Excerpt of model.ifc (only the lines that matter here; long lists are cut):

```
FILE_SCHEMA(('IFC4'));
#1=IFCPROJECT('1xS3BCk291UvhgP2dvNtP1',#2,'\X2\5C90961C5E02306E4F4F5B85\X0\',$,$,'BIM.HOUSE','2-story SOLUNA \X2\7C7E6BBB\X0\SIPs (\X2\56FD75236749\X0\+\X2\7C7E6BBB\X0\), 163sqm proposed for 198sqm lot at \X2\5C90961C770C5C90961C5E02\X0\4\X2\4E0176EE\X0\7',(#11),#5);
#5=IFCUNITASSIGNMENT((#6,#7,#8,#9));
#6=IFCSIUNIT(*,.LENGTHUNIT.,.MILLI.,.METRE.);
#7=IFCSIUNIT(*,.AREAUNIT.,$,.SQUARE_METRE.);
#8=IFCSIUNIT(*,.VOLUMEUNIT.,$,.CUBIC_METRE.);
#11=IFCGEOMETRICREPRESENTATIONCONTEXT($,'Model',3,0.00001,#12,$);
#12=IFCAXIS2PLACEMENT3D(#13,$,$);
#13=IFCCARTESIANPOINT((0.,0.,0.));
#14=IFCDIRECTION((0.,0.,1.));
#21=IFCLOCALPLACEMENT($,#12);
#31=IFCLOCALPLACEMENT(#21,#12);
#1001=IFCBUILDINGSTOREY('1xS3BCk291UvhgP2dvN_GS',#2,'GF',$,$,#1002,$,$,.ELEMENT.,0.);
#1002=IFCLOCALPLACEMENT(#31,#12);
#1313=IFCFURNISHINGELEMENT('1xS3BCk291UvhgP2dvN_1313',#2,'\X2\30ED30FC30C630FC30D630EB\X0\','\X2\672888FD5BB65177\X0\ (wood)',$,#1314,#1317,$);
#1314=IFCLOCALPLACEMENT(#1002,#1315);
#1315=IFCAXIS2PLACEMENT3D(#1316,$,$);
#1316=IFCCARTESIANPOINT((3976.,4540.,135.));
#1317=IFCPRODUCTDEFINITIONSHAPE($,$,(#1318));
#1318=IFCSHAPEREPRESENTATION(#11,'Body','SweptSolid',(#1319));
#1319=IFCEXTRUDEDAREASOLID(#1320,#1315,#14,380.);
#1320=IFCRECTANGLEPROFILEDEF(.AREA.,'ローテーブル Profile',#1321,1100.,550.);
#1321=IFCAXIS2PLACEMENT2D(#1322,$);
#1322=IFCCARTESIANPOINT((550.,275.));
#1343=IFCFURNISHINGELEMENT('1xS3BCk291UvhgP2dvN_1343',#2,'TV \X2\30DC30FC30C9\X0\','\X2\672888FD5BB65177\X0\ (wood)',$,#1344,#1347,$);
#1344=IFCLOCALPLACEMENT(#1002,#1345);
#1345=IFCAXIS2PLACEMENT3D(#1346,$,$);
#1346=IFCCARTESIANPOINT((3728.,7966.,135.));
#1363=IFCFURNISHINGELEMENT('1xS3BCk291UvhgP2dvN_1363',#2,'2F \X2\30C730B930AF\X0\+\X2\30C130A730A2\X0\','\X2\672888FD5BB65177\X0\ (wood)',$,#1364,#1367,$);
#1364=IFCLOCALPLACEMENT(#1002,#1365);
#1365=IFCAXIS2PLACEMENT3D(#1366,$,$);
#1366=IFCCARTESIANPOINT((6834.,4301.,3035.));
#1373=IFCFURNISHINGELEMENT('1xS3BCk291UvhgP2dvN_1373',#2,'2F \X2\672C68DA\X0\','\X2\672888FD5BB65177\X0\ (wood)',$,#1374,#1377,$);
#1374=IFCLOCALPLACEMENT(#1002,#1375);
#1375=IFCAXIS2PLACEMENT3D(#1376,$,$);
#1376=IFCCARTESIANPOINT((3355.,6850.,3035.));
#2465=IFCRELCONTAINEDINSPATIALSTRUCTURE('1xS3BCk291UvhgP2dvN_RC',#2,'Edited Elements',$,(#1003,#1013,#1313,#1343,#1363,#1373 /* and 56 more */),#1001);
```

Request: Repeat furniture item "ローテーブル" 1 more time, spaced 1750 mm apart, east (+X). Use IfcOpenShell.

```python
import numpy as np
import ifcopenshell
import ifcopenshell.api.geometry
import ifcopenshell.api.root
import ifcopenshell.util.element
import ifcopenshell.util.placement
import ifcopenshell.util.unit

model = ifcopenshell.open("model.ifc")
unit_scale = ifcopenshell.util.unit.calculate_unit_scale(model)


def reuse_history(source, copy):
    """copy_class also copies each property set's owner history, people and application; keep the originals."""
    for rel in copy.IsDefinedBy:
        if rel.is_a("IfcRelDefinesByProperties") and (history := rel.RelatingPropertyDefinition.OwnerHistory):
            rel.RelatingPropertyDefinition.OwnerHistory = source.OwnerHistory
            ifcopenshell.util.element.remove_deep2(model, history)


source = model.by_guid("1xS3BCk291UvhgP2dvN_1313")
base = ifcopenshell.util.placement.get_local_placement(source.ObjectPlacement)
step = np.array([1.0, 0.0, 0.0]) * 1.75 / unit_scale

for i in range(1, 2):
    copy = ifcopenshell.api.root.copy_class(model, product=source)
    copy.Representation = ifcopenshell.util.element.copy_deep(
        model, source.Representation, exclude=["IfcGeometricRepresentationContext", "IfcRepresentationMap"]
    )
    reuse_history(source, copy)
    matrix = base.copy()
    matrix[:3, 3] += i * step
    print("added at", matrix[:3, 3].round(3) + 0.0)
    ifcopenshell.api.geometry.edit_object_placement(model, product=copy, matrix=matrix, is_si=False)

model.write("model_rev.ifc")
```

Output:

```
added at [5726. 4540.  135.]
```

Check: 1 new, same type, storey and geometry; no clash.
